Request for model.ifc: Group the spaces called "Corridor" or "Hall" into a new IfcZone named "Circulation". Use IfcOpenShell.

First a look at what the model holds.

```python
import ifcopenshell

model = ifcopenshell.open("model.ifc")
print(model.schema)
seen = {}
for space in model.by_type("IfcSpace"):
    seen[space.LongName] = seen.get(space.LongName, 0) + 1
for name, count in sorted(seen.items(), key=str):
    print(count, "x", name)
print("zones:", [z.Name for z in model.by_type("IfcZone")][:20])
```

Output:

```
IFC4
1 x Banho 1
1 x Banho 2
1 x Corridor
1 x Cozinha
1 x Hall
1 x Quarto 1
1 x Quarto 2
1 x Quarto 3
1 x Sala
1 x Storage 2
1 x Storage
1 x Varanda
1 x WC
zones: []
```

```python
import ifcopenshell
import ifcopenshell.api.group
import ifcopenshell.api.root

model = ifcopenshell.open("model.ifc")

names = {"Corridor", "Hall"}
spaces = [s for s in model.by_type("IfcSpace") if s.LongName in names]

zone = ifcopenshell.api.root.create_entity(model, ifc_class="IfcZone", name="Circulation")
ifcopenshell.api.group.assign_group(model, products=spaces, group=zone)
print(len(spaces), "spaces in", zone.Name)

model.write("model_edited.ifc")
```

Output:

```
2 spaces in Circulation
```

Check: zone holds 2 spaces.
